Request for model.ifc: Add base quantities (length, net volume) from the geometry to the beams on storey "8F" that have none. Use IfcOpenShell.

First a look at what the model holds.

```python
import ifcopenshell
import ifcopenshell.util.element
import ifcopenshell.util.unit

model = ifcopenshell.open("model.ifc")
print(model.schema)
for unit_type in ("LENGTHUNIT", "AREAUNIT", "VOLUMEUNIT"):
    print(unit_type, ifcopenshell.util.unit.calculate_unit_scale(model, unit_type))
storey = next(s for s in model.by_type("IfcBuildingStorey") if s.Name == "8F")
beams = [e for e in ifcopenshell.util.element.get_decomposition(storey) if e.is_a("IfcBeam")]
for e in sorted(beams, key=lambda e: e.id()):
    print(e.id(), e.is_a(), e.Name, list(ifcopenshell.util.element.get_psets(e, qtos_only=True)), sep=" | ")
```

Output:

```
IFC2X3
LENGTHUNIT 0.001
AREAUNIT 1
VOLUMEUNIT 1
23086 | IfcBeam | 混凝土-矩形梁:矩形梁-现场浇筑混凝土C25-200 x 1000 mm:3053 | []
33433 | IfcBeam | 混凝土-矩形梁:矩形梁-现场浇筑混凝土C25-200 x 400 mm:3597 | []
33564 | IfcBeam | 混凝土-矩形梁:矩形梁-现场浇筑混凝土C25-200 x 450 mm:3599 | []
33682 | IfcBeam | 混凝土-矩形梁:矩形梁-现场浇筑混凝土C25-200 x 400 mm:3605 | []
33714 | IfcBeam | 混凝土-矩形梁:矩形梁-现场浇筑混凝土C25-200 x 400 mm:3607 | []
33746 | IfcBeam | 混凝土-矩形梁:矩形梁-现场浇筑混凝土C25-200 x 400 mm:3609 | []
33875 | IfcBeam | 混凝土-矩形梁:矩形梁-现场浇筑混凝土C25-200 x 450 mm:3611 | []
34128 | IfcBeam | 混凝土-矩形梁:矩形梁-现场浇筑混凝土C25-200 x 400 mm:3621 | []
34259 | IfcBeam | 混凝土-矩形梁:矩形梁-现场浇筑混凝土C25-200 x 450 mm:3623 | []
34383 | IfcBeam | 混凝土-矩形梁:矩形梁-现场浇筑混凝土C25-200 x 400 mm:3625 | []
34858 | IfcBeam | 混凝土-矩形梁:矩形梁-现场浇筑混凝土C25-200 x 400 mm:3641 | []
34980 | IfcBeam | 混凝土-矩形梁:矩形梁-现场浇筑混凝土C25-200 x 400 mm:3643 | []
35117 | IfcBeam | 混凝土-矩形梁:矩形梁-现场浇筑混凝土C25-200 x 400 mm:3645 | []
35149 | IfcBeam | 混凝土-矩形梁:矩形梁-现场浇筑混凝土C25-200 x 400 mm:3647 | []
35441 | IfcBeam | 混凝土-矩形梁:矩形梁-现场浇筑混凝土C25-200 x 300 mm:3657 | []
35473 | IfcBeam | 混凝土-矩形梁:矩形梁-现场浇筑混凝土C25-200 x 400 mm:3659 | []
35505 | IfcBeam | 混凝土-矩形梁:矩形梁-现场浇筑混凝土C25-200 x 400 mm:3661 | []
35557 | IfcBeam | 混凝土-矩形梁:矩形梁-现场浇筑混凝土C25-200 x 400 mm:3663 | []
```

```python
import ifcopenshell
import ifcopenshell.api.pset
import ifcopenshell.geom
import ifcopenshell.util.element
import ifcopenshell.util.shape
import ifcopenshell.util.unit

model = ifcopenshell.open("model.ifc")
unit_scale = ifcopenshell.util.unit.calculate_unit_scale(model)
volume_scale = ifcopenshell.util.unit.calculate_unit_scale(model, "VOLUMEUNIT")
settings = ifcopenshell.geom.settings()

storey = next(s for s in model.by_type("IfcBuildingStorey") if s.Name == "8F")
beams = [e for e in ifcopenshell.util.element.get_decomposition(storey) if e.is_a("IfcBeam")]

for e in sorted(beams, key=lambda e: e.id()):
    if ifcopenshell.util.element.get_psets(e, qtos_only=True, should_inherit=False):
        continue
    # Geometry comes back in metres, in the element's own axes.
    shape = ifcopenshell.geom.create_shape(settings, e)
    values = {
        "Length": ifcopenshell.util.shape.get_max_xyz(shape.geometry) / unit_scale,
        "NetVolume": ifcopenshell.util.shape.get_volume(shape.geometry) / volume_scale,
    }
    qto = ifcopenshell.api.pset.add_qto(model, product=e, name="BaseQuantities")
    ifcopenshell.api.pset.edit_qto(model, qto=qto, properties=values)
    print(e.id(), {k: round(v, 3) for k, v in values.items()})

model.write("model_rev.ifc")
```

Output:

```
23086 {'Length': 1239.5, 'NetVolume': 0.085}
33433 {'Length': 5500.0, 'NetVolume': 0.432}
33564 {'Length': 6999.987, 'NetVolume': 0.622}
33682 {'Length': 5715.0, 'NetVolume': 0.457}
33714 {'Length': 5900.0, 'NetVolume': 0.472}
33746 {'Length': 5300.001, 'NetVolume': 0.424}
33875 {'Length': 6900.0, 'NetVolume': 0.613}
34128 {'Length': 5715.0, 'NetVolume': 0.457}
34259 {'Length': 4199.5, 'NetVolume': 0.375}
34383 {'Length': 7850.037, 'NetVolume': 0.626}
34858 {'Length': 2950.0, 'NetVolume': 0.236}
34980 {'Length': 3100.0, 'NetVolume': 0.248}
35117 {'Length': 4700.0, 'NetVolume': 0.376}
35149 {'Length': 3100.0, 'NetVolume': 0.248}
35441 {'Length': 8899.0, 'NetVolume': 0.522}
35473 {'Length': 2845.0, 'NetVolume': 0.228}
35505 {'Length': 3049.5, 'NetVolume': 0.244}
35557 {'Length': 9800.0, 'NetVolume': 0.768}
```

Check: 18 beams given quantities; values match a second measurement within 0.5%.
